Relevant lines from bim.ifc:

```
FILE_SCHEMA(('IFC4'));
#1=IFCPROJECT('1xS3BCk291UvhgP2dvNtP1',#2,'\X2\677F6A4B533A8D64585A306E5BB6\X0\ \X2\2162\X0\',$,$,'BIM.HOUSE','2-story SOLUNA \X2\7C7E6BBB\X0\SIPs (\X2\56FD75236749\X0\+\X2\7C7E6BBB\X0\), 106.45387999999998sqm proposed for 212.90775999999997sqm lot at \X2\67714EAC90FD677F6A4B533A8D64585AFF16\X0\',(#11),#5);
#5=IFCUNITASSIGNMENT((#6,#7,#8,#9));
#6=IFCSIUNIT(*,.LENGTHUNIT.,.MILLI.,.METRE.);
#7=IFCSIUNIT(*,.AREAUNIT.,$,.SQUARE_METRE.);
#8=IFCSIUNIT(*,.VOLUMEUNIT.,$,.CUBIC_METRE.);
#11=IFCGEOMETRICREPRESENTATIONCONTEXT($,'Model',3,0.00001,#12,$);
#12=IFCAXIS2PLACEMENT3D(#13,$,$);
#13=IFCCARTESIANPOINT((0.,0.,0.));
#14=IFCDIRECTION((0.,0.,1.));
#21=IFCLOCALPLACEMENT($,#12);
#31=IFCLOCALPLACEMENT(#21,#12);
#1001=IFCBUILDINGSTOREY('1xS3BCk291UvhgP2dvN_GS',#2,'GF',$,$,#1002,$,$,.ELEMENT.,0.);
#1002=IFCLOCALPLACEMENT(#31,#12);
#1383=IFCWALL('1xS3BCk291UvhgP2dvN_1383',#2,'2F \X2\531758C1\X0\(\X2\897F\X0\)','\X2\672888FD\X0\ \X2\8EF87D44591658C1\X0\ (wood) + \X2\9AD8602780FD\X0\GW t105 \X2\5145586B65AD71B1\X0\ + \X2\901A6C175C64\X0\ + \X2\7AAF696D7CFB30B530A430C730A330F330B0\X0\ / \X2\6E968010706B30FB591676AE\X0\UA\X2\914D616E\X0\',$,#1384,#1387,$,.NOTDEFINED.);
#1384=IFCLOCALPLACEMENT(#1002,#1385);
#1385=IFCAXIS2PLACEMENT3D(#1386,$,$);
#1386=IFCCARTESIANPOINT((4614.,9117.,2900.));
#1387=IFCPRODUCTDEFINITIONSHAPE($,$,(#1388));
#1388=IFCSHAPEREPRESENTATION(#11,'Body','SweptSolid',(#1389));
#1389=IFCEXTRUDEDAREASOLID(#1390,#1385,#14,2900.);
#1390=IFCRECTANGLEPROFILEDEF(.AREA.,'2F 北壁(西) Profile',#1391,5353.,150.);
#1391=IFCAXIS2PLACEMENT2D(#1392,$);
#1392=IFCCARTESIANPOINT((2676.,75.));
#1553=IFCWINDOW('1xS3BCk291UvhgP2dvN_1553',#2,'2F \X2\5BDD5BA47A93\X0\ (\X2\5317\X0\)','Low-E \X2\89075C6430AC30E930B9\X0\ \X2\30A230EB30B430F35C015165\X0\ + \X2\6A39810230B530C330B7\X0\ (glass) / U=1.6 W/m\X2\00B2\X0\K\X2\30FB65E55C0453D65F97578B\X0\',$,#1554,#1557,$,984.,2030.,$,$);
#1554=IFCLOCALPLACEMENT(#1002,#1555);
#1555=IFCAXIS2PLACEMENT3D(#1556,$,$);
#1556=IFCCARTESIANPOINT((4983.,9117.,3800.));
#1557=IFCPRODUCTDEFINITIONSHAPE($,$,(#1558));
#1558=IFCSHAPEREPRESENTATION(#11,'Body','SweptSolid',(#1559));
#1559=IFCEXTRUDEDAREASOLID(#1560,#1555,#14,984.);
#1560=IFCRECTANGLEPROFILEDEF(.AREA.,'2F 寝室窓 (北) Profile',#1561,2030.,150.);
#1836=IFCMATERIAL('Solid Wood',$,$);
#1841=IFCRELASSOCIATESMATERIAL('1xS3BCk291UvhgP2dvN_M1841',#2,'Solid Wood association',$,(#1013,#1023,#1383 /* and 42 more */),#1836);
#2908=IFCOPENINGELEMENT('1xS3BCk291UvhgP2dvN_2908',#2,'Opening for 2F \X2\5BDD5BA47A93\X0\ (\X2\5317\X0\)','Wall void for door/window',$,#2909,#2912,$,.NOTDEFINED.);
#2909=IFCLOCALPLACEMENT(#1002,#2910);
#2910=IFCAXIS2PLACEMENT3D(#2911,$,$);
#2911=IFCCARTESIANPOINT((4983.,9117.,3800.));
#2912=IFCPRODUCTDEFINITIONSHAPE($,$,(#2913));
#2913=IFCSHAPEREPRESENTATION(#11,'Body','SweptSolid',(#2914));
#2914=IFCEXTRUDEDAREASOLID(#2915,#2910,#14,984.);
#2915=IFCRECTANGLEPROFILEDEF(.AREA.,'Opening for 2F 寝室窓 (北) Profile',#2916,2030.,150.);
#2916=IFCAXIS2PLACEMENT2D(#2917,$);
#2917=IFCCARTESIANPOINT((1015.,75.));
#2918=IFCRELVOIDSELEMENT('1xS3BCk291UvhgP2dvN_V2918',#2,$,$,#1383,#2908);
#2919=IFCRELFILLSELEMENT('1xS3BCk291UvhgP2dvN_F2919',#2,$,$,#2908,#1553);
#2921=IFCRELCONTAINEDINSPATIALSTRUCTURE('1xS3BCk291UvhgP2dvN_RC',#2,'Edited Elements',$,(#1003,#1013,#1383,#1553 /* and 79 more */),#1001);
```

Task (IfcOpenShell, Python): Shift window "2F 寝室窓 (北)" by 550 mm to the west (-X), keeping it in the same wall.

```python
import ifcopenshell
import ifcopenshell.api.geometry
import ifcopenshell.util.placement
import ifcopenshell.util.unit

model = ifcopenshell.open("bim.ifc")
unit_scale = ifcopenshell.util.unit.calculate_unit_scale(model)

window = model.by_guid("1xS3BCk291UvhgP2dvN_1553")
opening = window.FillsVoids[0].RelatingOpeningElement
wall = opening.VoidsElements[0].RelatingBuildingElement

wall_matrix = ifcopenshell.util.placement.get_local_placement(wall.ObjectPlacement)
shift = wall_matrix[:3, 0] * -0.55 / unit_scale
before = ifcopenshell.util.placement.get_local_placement(window.ObjectPlacement)[:3, 3].copy()

# The window is not placed relative to its opening, so move both.
for product in (opening, window):
    matrix = ifcopenshell.util.placement.get_local_placement(product.ObjectPlacement)
    matrix[:3, 3] += shift
    ifcopenshell.api.geometry.edit_object_placement(model, product=product, matrix=matrix, is_si=False)

after = ifcopenshell.util.placement.get_local_placement(window.ObjectPlacement)[:3, 3]
print("window moved by", (after - before).round(3) + 0.0)

model.write("bim_updated.ifc")
```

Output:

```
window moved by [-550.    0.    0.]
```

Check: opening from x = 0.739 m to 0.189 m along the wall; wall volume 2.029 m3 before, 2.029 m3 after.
